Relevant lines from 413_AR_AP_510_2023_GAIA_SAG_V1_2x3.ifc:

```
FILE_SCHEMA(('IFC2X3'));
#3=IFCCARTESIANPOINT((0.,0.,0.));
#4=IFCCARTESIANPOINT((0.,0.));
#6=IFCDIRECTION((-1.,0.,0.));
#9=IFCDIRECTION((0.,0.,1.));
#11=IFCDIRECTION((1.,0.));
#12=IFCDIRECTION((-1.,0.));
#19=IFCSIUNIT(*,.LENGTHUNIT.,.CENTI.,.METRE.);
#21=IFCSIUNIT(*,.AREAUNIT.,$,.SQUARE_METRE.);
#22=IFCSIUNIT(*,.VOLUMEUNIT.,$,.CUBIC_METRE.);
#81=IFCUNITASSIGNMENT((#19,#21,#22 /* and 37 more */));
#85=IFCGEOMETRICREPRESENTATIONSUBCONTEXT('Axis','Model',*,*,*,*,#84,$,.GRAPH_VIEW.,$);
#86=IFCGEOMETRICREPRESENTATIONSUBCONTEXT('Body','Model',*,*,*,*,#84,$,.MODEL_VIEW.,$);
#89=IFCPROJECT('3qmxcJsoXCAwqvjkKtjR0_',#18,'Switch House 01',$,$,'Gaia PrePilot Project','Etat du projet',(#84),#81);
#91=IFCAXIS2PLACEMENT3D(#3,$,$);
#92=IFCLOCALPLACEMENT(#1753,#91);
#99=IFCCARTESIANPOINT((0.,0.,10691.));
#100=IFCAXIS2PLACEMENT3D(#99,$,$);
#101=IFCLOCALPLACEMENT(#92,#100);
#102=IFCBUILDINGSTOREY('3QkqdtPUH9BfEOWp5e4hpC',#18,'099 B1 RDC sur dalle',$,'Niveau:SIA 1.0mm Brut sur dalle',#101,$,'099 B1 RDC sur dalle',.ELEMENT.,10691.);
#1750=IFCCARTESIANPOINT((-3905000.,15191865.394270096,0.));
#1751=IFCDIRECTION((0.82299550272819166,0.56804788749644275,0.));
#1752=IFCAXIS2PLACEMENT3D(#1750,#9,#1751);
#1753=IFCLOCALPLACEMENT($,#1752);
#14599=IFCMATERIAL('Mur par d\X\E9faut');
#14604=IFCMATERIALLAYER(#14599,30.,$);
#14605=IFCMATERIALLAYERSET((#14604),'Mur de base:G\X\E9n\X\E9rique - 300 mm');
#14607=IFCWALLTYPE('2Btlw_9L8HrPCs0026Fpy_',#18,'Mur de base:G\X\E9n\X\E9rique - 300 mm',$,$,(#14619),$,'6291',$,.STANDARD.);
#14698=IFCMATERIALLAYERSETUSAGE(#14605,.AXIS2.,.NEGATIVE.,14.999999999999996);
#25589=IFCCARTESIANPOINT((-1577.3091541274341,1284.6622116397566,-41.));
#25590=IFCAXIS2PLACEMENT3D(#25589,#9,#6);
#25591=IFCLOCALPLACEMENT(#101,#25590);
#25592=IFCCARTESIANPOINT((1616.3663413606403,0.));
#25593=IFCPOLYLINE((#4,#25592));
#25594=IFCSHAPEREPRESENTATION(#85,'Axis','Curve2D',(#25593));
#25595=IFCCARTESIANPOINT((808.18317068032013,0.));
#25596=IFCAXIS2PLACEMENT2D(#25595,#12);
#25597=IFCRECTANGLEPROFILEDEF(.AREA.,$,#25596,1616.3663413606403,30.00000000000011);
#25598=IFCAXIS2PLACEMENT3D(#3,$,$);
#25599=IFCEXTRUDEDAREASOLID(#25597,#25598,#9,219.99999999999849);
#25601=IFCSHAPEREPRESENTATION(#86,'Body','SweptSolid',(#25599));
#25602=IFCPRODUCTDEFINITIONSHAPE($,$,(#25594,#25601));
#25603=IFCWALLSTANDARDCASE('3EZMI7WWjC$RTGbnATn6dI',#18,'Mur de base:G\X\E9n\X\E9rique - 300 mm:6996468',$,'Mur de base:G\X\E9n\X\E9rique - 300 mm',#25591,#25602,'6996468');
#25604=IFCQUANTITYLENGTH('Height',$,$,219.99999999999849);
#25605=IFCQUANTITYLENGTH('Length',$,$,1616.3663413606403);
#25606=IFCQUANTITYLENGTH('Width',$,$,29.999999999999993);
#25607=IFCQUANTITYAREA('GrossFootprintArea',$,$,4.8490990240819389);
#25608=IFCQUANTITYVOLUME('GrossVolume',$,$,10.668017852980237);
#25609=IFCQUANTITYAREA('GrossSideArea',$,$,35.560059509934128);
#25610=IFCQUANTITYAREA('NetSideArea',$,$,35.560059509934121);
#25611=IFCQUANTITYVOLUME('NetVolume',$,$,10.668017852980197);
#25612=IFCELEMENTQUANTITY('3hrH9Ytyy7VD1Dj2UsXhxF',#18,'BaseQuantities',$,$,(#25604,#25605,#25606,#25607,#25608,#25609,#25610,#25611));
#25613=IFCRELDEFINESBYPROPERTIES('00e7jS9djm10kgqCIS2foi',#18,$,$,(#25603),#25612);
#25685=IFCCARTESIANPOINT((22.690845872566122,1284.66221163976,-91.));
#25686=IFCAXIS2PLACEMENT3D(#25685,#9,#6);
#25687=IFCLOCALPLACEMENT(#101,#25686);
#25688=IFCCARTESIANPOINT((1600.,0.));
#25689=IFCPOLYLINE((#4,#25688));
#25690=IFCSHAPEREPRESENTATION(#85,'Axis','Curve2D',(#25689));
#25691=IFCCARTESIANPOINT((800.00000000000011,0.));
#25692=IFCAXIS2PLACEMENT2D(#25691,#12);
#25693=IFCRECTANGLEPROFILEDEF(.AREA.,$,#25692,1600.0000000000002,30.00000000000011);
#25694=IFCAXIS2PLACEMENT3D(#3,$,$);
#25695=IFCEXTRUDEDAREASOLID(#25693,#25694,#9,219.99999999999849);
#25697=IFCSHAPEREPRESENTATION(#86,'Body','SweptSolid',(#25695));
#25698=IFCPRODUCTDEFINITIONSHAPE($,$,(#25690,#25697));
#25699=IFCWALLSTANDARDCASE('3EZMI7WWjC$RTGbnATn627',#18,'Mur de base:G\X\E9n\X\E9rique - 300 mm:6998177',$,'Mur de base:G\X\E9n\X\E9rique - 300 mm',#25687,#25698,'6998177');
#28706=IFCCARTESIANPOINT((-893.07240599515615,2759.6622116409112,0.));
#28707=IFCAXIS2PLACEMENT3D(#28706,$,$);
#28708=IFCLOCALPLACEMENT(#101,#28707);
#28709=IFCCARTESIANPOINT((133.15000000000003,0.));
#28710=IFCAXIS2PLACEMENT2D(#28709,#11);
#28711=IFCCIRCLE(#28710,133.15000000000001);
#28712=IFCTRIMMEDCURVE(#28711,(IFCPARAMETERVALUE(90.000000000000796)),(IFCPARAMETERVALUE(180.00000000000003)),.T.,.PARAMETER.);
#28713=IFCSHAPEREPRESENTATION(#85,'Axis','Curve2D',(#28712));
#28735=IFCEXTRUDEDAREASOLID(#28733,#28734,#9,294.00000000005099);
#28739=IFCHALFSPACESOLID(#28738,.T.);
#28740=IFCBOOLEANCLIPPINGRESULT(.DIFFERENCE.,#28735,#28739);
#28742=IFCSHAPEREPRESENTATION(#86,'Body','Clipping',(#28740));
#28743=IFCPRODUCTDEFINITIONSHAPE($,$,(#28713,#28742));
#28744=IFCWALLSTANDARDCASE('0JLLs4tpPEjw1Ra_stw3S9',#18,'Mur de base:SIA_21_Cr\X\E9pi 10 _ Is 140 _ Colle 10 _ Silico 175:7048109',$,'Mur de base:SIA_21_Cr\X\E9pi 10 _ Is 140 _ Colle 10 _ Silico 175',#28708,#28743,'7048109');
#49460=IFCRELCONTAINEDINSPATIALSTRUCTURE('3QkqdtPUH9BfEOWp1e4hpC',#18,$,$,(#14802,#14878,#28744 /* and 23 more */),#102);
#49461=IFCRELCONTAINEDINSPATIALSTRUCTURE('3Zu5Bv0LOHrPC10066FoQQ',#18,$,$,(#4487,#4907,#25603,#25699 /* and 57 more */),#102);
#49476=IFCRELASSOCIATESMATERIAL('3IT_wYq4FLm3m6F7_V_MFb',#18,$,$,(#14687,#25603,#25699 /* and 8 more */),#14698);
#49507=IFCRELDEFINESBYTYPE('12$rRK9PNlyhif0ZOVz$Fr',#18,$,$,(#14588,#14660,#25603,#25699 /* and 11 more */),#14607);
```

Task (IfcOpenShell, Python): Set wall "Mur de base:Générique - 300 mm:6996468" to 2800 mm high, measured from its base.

```python
import ifcopenshell
import ifcopenshell.api.pset
import ifcopenshell.geom
import ifcopenshell.util.element
import ifcopenshell.util.representation
import ifcopenshell.util.shape
import ifcopenshell.util.unit

model = ifcopenshell.open("413_AR_AP_510_2023_GAIA_SAG_V1_2x3.ifc")
unit_scale = ifcopenshell.util.unit.calculate_unit_scale(model)
area_scale = ifcopenshell.util.unit.calculate_unit_scale(model, "AREAUNIT")
volume_scale = ifcopenshell.util.unit.calculate_unit_scale(model, "VOLUMEUNIT")
settings = ifcopenshell.geom.settings()


def volume(element):
    """Net volume in cubic metres, openings subtracted."""
    shape = ifcopenshell.geom.create_shape(settings, element)
    return ifcopenshell.util.shape.get_volume(shape.geometry)


wall = model.by_guid("3EZMI7WWjC$RTGbnATn6dI")
before = volume(wall)

body = ifcopenshell.util.representation.get_representation(wall, "Model", "Body")
solid = body.Items[0]
old_height = solid.Depth
solid.Depth = 2.8 / unit_scale
after = volume(wall)
thickness = 0.3  # wall thickness in metres

# Update the stored height, areas and volumes.
qto = model.by_id(ifcopenshell.util.element.get_pset(wall, "BaseQuantities", should_inherit=False)["id"])
ifcopenshell.api.pset.edit_qto(model, qto=qto, properties={
    "Height": solid.Depth,
    "GrossVolume": ifcopenshell.util.element.get_pset(wall, "BaseQuantities", "GrossVolume") * solid.Depth / old_height,
    "GrossSideArea": ifcopenshell.util.element.get_pset(wall, "BaseQuantities", "GrossSideArea") * solid.Depth / old_height,
    "NetSideArea": after / thickness / area_scale,
    "NetVolume": after / volume_scale,
})

print(f"height {old_height:g} -> {solid.Depth:g}, volume {before:.3f} -> {after:.3f} m3")

model.write("413_AR_AP_510_2023_GAIA_SAG_V1_2x3_edited.ifc")
```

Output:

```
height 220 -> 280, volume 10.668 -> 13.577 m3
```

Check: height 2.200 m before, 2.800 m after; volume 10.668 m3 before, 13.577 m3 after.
